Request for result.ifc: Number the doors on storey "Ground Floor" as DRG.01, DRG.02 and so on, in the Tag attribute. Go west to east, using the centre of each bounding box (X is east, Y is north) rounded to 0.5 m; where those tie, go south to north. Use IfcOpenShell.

First a look at what the model holds.

```python
import ifcopenshell
import ifcopenshell.util.element
import ifcopenshell.util.placement

model = ifcopenshell.open("result.ifc")
print(model.schema)
storey = next(s for s in model.by_type("IfcBuildingStorey") if s.Name == "Ground Floor")
doors = [e for e in ifcopenshell.util.element.get_decomposition(storey) if e.is_a("IfcDoor")]
for e in sorted(doors, key=lambda e: e.id()):
    origin = ifcopenshell.util.placement.get_local_placement(e.ObjectPlacement)[:3, 3]
    print(e.id(), e.Tag, e.Name, origin.round(2) + 0.0, sep=" | ")
```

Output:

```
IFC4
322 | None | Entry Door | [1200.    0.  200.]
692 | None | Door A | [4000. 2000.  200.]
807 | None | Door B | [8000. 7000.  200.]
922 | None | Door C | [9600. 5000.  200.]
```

```python
import ifcopenshell
import ifcopenshell.geom
import ifcopenshell.util.element
import ifcopenshell.util.shape

model = ifcopenshell.open("result.ifc")
settings = ifcopenshell.geom.settings()
settings.set("use-world-coords", True)


def centre(element):
    shape = ifcopenshell.geom.create_shape(settings, element)
    return ifcopenshell.util.shape.get_bbox_centroid(shape.geometry)


storey = next(s for s in model.by_type("IfcBuildingStorey") if s.Name == "Ground Floor")
doors = [e for e in ifcopenshell.util.element.get_decomposition(storey) if e.is_a("IfcDoor")]

# Insertion points can sit at a corner or the storey origin, so sort by the geometry (in metres).
centres = {e: centre(e) for e in doors}
doors.sort(key=lambda e: (round(centres[e][0] / 0.5), centres[e][1]))

for i, e in enumerate(doors, start=1):
    number = f"DRG.{i:02d}"
    e.Tag = number
    print(e.id(), number)

model.write("result_rev.ifc")
```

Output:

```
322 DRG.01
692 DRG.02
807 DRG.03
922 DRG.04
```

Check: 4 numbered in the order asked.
